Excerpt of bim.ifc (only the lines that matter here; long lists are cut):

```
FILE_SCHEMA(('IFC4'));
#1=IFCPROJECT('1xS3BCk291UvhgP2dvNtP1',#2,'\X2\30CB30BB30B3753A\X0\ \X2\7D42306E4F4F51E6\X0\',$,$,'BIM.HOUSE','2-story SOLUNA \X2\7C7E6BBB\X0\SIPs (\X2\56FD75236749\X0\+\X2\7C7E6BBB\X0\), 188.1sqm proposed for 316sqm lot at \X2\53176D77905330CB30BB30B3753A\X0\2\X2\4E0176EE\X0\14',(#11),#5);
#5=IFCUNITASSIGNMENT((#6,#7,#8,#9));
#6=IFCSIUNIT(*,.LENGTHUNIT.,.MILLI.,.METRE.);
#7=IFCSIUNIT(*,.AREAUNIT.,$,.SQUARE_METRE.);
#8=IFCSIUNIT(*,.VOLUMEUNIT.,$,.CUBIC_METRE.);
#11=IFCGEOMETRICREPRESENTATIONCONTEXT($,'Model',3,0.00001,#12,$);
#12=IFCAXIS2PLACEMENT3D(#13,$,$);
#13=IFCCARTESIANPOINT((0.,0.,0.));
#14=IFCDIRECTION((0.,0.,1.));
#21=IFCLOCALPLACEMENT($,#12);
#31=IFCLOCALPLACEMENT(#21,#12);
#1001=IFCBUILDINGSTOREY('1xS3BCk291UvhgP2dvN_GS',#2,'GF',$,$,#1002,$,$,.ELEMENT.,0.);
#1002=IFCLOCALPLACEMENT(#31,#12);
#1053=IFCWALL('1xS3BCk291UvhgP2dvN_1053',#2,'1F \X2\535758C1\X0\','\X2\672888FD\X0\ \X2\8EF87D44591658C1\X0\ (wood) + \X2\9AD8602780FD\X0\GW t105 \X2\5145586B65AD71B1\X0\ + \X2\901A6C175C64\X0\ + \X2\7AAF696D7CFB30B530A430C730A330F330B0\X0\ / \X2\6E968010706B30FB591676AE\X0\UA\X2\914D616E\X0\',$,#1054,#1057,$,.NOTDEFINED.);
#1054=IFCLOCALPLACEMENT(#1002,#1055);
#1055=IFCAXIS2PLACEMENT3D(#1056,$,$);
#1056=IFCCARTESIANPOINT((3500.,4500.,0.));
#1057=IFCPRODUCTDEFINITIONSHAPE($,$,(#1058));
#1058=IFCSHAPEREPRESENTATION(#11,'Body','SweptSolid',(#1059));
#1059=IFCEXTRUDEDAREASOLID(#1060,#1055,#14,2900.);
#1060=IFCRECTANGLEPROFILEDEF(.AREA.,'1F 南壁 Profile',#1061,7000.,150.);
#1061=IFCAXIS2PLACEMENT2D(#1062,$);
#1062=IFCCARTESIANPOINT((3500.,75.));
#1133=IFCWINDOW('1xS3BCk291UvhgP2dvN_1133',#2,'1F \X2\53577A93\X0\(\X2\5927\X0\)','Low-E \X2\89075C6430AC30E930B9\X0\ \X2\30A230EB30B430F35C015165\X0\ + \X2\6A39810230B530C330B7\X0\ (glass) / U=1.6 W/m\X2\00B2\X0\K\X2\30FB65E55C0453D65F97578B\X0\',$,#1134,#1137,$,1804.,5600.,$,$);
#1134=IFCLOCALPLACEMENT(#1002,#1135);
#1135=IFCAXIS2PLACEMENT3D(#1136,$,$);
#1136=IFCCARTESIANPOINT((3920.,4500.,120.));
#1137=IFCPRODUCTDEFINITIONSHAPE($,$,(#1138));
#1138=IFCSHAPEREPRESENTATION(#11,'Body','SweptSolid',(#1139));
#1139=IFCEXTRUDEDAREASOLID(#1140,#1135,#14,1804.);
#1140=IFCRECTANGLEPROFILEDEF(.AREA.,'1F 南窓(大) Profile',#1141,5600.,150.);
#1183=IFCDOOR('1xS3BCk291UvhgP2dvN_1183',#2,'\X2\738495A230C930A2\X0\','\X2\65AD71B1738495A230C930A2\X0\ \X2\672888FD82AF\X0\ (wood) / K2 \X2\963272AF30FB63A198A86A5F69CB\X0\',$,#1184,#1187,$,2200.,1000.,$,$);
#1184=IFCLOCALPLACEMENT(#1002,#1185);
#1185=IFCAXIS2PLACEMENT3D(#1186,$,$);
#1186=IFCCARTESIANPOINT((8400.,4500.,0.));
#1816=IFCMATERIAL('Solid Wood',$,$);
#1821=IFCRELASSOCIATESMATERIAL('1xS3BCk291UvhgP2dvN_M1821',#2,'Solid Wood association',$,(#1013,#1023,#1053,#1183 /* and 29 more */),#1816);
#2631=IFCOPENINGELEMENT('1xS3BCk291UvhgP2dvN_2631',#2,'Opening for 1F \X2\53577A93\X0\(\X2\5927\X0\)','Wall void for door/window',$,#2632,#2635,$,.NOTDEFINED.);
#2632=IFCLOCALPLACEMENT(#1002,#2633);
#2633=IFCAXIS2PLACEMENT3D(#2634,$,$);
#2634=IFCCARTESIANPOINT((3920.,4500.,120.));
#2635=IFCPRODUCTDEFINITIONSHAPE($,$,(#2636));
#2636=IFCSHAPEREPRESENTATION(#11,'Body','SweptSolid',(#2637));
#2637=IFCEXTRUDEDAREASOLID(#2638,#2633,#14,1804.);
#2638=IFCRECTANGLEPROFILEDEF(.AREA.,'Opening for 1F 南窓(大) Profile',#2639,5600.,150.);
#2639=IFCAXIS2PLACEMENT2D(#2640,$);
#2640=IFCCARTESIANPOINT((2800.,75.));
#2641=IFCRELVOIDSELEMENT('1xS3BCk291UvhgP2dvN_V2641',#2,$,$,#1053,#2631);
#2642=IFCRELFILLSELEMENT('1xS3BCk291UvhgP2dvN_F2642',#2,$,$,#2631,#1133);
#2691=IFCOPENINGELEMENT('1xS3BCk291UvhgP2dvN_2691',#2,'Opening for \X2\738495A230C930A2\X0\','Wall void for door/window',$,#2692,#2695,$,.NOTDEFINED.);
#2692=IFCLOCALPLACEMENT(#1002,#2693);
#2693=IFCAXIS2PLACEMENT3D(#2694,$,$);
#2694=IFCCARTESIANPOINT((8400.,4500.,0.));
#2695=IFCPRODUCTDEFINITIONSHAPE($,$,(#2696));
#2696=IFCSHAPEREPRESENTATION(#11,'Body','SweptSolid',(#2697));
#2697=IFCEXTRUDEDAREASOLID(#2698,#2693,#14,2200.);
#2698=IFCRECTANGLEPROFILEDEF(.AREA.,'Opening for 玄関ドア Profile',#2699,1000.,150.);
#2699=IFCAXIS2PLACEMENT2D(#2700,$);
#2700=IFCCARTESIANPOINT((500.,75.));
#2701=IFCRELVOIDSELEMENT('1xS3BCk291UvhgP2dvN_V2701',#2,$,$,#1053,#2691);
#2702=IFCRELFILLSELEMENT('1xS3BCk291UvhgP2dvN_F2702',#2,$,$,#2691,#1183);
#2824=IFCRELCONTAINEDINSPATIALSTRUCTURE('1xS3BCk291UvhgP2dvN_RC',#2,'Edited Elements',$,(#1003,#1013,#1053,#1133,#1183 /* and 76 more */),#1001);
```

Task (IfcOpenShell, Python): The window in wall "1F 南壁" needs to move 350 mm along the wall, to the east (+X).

```python
import ifcopenshell
import ifcopenshell.api.geometry
import ifcopenshell.util.placement

model = ifcopenshell.open("bim.ifc")

window = model.by_guid("1xS3BCk291UvhgP2dvN_1133")
opening = window.FillsVoids[0].RelatingOpeningElement
wall = opening.VoidsElements[0].RelatingBuildingElement

wall_matrix = ifcopenshell.util.placement.get_local_placement(wall.ObjectPlacement)
shift = wall_matrix[:3, 0] * 350.0
before = ifcopenshell.util.placement.get_local_placement(window.ObjectPlacement)[:3, 3].copy()

# The window is not placed relative to its opening, so move both.
for product in (opening, window):
    matrix = ifcopenshell.util.placement.get_local_placement(product.ObjectPlacement)
    matrix[:3, 3] += shift
    ifcopenshell.api.geometry.edit_object_placement(model, product=product, matrix=matrix, is_si=False)

after = ifcopenshell.util.placement.get_local_placement(window.ObjectPlacement)[:3, 3]
print("window moved by", (after - before).round(3) + 0.0)

model.write("bim_rev.ifc")
```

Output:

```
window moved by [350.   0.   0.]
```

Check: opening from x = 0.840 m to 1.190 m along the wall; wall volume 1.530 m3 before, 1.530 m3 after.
